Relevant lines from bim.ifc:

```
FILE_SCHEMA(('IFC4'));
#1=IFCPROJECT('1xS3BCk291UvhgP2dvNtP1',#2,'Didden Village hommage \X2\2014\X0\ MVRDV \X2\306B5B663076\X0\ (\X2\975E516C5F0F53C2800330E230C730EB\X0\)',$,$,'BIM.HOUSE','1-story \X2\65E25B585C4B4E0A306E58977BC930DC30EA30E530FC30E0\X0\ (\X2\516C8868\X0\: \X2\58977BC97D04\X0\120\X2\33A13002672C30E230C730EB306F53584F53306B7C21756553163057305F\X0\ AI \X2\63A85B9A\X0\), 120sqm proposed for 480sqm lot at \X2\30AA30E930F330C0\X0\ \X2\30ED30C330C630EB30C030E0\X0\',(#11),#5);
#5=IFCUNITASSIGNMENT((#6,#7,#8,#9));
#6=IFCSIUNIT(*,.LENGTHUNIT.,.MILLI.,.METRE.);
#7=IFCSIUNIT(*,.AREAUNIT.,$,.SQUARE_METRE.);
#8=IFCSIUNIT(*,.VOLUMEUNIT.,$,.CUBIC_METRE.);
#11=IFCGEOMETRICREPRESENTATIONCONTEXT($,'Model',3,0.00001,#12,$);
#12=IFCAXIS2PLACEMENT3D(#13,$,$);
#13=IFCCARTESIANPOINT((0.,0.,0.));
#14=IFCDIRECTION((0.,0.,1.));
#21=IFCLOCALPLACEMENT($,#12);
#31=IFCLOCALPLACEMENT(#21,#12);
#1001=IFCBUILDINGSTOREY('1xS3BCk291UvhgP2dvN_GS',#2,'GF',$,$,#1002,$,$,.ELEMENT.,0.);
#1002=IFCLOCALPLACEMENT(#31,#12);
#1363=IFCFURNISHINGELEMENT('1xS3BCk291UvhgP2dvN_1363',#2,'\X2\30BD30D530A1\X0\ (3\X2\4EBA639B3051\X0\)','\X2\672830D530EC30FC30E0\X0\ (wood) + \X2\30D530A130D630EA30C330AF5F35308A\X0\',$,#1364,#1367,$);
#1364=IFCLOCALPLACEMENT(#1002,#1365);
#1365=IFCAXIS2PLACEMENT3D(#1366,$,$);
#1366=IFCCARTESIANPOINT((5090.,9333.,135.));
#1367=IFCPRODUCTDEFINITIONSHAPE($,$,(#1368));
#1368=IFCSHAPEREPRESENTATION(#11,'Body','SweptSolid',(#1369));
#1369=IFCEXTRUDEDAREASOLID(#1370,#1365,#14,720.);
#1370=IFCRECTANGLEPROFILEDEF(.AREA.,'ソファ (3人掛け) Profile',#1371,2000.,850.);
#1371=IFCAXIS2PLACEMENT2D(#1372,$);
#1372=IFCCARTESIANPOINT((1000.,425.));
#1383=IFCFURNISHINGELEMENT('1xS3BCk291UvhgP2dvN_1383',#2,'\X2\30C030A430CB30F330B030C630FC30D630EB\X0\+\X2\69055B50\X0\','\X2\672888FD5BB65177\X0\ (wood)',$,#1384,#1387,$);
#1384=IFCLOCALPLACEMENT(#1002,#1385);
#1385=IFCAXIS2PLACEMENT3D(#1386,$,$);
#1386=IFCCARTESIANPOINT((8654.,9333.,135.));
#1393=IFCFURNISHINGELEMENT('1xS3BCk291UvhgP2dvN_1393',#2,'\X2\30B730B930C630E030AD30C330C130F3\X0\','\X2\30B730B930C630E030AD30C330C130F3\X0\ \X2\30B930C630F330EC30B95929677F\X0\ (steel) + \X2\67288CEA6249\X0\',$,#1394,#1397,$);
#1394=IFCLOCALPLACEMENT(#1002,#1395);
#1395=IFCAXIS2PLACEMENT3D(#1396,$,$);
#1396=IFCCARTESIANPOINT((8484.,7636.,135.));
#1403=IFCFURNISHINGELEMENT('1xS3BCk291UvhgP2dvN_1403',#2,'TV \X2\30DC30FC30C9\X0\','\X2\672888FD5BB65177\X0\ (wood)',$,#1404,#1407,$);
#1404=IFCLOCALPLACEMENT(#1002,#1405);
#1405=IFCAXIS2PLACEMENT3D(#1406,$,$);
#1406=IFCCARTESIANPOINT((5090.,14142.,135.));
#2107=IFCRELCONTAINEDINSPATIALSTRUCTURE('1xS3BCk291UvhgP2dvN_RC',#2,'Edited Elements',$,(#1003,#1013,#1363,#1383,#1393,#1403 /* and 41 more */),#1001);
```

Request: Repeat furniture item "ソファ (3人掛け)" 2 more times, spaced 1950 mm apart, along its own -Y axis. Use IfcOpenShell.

```python
import ifcopenshell
import ifcopenshell.api.geometry
import ifcopenshell.api.root
import ifcopenshell.util.element
import ifcopenshell.util.placement

model = ifcopenshell.open("bim.ifc")


def reuse_history(source, copy):
    """copy_class also copies each property set's owner history, people and application; keep the originals."""
    for rel in copy.IsDefinedBy:
        if rel.is_a("IfcRelDefinesByProperties") and (history := rel.RelatingPropertyDefinition.OwnerHistory):
            rel.RelatingPropertyDefinition.OwnerHistory = source.OwnerHistory
            ifcopenshell.util.element.remove_deep2(model, history)


source = model.by_guid("1xS3BCk291UvhgP2dvN_1363")
base = ifcopenshell.util.placement.get_local_placement(source.ObjectPlacement)
step = -base[:3, 1] * 1950.0

for i in range(1, 3):
    copy = ifcopenshell.api.root.copy_class(model, product=source)
    copy.Representation = ifcopenshell.util.element.copy_deep(
        model, source.Representation, exclude=["IfcGeometricRepresentationContext", "IfcRepresentationMap"]
    )
    reuse_history(source, copy)
    matrix = base.copy()
    matrix[:3, 3] += i * step
    print("added at", matrix[:3, 3].round(3) + 0.0)
    ifcopenshell.api.geometry.edit_object_placement(model, product=copy, matrix=matrix, is_si=False)

model.write("bim_rev.ifc")
```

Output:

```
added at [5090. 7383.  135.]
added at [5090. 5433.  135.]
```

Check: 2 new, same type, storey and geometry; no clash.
